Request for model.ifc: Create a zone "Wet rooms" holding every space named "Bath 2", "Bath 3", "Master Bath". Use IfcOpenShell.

First a look at what the model holds.

```python
import ifcopenshell

model = ifcopenshell.open("model.ifc")
print(model.schema)
seen = {}
for space in model.by_type("IfcSpace"):
    seen[space.LongName] = seen.get(space.LongName, 0) + 1
for name, count in sorted(seen.items(), key=str):
    print(count, "x", name)
print("zones:", [z.Name for z in model.by_type("IfcZone")][:20])
```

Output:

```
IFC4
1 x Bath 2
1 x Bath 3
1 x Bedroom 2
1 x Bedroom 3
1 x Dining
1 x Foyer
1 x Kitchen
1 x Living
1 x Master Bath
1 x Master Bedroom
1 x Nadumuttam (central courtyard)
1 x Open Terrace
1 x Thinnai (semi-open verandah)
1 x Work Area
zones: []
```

```python
import ifcopenshell
import ifcopenshell.api.group
import ifcopenshell.api.root

model = ifcopenshell.open("model.ifc")

names = {"Bath 2", "Bath 3", "Master Bath"}
spaces = [s for s in model.by_type("IfcSpace") if s.LongName in names]

zone = ifcopenshell.api.root.create_entity(model, ifc_class="IfcZone", name="Wet rooms")
ifcopenshell.api.group.assign_group(model, products=spaces, group=zone)
print(len(spaces), "spaces in", zone.Name)

model.write("model_edited.ifc")
```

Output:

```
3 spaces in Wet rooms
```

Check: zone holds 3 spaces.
